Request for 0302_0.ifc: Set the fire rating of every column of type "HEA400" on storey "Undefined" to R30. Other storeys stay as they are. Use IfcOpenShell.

First a look at what the model holds.

```python
import ifcopenshell
import ifcopenshell.util.element

model = ifcopenshell.open("0302_0.ifc")
print(model.schema)
storey = next(s for s in model.by_type("IfcBuildingStorey") if s.Name == "Undefined")
columns = [e for e in ifcopenshell.util.element.get_decomposition(storey) if e.is_a("IfcColumn")]
seen = {}
for e in columns:
    element_type = ifcopenshell.util.element.get_type(e)
    key = (element_type.Name if element_type != e and element_type else None, ifcopenshell.util.element.get_pset(e, "Pset_ColumnCommon", "FireRating"))
    seen[key] = seen.get(key, 0) + 1
for (name, value), count in sorted(seen.items(), key=str):
    print(count, "x", name, "|", value)
```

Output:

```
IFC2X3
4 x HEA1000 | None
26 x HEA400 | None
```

```python
import ifcopenshell
import ifcopenshell.api.pset
import ifcopenshell.util.element

model = ifcopenshell.open("0302_0.ifc")

storey = next(s for s in model.by_type("IfcBuildingStorey") if s.Name == "Undefined")
columns = [e for e in ifcopenshell.util.element.get_decomposition(storey) if e.is_a("IfcColumn")]

count = 0
for e in columns:
    element_type = ifcopenshell.util.element.get_type(e)
    if element_type in (None, e) or element_type.Name != "HEA400":
        continue
    found = ifcopenshell.util.element.get_pset(e, "Pset_ColumnCommon", should_inherit=False)
    if found:
        pset = model.by_id(found["id"])
        if len(ifcopenshell.util.element.get_elements_by_pset(pset)) > 1:
            pset = ifcopenshell.api.pset.unshare_pset(model, products=[e], pset=pset)[0]
    else:
        pset = ifcopenshell.api.pset.add_pset(model, product=e, name="Pset_ColumnCommon")
    ifcopenshell.api.pset.edit_pset(model, pset=pset, properties={"FireRating": "R30"})
    count += 1

print(count, "columns updated")

model.write("0302_0_v2.ifc")
```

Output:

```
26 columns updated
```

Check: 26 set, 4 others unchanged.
